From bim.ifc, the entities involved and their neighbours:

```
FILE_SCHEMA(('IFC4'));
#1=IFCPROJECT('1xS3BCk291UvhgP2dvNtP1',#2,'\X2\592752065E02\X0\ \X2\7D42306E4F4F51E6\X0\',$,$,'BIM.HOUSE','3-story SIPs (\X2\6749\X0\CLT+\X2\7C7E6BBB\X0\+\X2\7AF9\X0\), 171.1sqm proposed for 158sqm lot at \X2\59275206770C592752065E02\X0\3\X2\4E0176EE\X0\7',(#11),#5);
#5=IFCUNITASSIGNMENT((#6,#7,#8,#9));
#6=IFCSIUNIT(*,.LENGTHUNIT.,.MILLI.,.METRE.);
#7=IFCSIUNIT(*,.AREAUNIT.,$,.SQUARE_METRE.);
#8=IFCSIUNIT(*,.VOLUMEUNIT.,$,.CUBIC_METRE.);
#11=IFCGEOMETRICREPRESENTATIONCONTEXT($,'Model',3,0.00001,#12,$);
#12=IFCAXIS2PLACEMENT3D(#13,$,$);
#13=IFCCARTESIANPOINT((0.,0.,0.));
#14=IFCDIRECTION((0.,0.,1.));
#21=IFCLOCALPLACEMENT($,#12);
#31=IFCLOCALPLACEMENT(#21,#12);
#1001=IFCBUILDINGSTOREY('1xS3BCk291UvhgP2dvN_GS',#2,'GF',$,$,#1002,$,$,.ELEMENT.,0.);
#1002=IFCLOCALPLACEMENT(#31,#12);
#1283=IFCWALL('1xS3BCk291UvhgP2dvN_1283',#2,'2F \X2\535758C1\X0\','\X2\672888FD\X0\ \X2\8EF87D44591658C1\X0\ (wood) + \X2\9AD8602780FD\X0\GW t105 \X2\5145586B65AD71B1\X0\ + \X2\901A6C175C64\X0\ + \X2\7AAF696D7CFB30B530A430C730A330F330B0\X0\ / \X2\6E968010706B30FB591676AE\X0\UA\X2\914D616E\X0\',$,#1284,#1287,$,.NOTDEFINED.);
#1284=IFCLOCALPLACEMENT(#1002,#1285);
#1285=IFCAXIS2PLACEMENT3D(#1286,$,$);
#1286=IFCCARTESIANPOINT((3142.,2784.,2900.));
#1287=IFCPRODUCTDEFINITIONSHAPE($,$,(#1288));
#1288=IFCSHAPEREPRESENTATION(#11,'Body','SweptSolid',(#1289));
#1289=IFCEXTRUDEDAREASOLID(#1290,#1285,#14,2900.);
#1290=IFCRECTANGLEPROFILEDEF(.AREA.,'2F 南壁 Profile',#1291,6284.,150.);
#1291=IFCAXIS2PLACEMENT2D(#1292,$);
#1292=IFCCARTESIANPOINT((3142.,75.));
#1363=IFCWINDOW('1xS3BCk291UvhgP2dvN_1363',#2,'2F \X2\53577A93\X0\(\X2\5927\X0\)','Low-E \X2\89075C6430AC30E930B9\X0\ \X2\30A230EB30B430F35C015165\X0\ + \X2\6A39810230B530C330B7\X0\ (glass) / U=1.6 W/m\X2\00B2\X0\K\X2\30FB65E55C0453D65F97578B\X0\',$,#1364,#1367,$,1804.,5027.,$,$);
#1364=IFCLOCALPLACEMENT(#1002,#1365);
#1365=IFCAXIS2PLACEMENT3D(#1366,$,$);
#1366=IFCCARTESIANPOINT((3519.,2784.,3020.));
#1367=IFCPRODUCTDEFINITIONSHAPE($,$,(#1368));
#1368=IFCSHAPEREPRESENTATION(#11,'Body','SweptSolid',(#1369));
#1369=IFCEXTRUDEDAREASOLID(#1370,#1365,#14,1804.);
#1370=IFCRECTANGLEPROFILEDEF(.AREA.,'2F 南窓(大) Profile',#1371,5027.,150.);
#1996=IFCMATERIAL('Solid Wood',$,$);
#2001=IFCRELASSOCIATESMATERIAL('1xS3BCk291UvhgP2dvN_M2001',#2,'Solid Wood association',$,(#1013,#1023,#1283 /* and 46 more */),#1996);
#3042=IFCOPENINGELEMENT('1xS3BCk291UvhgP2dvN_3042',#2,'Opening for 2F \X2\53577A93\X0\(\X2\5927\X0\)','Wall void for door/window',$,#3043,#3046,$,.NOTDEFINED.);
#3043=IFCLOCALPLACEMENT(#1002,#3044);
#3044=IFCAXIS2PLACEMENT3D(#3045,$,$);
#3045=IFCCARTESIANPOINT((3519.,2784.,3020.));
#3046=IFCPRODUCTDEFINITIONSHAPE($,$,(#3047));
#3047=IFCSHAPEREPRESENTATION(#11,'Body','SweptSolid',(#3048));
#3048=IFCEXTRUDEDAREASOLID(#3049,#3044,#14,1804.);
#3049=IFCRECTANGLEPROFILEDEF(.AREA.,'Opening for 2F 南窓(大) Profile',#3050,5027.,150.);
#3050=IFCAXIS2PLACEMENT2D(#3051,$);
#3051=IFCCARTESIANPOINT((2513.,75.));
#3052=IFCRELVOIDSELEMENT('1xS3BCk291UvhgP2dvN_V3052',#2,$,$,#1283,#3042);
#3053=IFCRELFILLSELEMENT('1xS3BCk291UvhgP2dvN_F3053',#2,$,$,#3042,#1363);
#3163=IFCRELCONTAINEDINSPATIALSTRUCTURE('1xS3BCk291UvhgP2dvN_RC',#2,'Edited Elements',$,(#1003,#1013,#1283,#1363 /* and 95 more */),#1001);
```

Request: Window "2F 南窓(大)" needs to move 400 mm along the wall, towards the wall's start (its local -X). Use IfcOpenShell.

```python
import ifcopenshell
import ifcopenshell.api.geometry
import ifcopenshell.util.placement

model = ifcopenshell.open("bim.ifc")

window = model.by_guid("1xS3BCk291UvhgP2dvN_1363")
opening = window.FillsVoids[0].RelatingOpeningElement
wall = opening.VoidsElements[0].RelatingBuildingElement

wall_matrix = ifcopenshell.util.placement.get_local_placement(wall.ObjectPlacement)
shift = wall_matrix[:3, 0] * -400.0
before = ifcopenshell.util.placement.get_local_placement(window.ObjectPlacement)[:3, 3].copy()

# The window is not placed relative to its opening, so move both.
for product in (opening, window):
    matrix = ifcopenshell.util.placement.get_local_placement(product.ObjectPlacement)
    matrix[:3, 3] += shift
    ifcopenshell.api.geometry.edit_object_placement(model, product=product, matrix=matrix, is_si=False)

after = ifcopenshell.util.placement.get_local_placement(window.ObjectPlacement)[:3, 3]
print("window moved by", (after - before).round(3) + 0.0)

model.write("bim_edited.ifc")
```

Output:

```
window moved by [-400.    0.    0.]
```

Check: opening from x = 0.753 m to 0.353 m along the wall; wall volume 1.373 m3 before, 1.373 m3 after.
